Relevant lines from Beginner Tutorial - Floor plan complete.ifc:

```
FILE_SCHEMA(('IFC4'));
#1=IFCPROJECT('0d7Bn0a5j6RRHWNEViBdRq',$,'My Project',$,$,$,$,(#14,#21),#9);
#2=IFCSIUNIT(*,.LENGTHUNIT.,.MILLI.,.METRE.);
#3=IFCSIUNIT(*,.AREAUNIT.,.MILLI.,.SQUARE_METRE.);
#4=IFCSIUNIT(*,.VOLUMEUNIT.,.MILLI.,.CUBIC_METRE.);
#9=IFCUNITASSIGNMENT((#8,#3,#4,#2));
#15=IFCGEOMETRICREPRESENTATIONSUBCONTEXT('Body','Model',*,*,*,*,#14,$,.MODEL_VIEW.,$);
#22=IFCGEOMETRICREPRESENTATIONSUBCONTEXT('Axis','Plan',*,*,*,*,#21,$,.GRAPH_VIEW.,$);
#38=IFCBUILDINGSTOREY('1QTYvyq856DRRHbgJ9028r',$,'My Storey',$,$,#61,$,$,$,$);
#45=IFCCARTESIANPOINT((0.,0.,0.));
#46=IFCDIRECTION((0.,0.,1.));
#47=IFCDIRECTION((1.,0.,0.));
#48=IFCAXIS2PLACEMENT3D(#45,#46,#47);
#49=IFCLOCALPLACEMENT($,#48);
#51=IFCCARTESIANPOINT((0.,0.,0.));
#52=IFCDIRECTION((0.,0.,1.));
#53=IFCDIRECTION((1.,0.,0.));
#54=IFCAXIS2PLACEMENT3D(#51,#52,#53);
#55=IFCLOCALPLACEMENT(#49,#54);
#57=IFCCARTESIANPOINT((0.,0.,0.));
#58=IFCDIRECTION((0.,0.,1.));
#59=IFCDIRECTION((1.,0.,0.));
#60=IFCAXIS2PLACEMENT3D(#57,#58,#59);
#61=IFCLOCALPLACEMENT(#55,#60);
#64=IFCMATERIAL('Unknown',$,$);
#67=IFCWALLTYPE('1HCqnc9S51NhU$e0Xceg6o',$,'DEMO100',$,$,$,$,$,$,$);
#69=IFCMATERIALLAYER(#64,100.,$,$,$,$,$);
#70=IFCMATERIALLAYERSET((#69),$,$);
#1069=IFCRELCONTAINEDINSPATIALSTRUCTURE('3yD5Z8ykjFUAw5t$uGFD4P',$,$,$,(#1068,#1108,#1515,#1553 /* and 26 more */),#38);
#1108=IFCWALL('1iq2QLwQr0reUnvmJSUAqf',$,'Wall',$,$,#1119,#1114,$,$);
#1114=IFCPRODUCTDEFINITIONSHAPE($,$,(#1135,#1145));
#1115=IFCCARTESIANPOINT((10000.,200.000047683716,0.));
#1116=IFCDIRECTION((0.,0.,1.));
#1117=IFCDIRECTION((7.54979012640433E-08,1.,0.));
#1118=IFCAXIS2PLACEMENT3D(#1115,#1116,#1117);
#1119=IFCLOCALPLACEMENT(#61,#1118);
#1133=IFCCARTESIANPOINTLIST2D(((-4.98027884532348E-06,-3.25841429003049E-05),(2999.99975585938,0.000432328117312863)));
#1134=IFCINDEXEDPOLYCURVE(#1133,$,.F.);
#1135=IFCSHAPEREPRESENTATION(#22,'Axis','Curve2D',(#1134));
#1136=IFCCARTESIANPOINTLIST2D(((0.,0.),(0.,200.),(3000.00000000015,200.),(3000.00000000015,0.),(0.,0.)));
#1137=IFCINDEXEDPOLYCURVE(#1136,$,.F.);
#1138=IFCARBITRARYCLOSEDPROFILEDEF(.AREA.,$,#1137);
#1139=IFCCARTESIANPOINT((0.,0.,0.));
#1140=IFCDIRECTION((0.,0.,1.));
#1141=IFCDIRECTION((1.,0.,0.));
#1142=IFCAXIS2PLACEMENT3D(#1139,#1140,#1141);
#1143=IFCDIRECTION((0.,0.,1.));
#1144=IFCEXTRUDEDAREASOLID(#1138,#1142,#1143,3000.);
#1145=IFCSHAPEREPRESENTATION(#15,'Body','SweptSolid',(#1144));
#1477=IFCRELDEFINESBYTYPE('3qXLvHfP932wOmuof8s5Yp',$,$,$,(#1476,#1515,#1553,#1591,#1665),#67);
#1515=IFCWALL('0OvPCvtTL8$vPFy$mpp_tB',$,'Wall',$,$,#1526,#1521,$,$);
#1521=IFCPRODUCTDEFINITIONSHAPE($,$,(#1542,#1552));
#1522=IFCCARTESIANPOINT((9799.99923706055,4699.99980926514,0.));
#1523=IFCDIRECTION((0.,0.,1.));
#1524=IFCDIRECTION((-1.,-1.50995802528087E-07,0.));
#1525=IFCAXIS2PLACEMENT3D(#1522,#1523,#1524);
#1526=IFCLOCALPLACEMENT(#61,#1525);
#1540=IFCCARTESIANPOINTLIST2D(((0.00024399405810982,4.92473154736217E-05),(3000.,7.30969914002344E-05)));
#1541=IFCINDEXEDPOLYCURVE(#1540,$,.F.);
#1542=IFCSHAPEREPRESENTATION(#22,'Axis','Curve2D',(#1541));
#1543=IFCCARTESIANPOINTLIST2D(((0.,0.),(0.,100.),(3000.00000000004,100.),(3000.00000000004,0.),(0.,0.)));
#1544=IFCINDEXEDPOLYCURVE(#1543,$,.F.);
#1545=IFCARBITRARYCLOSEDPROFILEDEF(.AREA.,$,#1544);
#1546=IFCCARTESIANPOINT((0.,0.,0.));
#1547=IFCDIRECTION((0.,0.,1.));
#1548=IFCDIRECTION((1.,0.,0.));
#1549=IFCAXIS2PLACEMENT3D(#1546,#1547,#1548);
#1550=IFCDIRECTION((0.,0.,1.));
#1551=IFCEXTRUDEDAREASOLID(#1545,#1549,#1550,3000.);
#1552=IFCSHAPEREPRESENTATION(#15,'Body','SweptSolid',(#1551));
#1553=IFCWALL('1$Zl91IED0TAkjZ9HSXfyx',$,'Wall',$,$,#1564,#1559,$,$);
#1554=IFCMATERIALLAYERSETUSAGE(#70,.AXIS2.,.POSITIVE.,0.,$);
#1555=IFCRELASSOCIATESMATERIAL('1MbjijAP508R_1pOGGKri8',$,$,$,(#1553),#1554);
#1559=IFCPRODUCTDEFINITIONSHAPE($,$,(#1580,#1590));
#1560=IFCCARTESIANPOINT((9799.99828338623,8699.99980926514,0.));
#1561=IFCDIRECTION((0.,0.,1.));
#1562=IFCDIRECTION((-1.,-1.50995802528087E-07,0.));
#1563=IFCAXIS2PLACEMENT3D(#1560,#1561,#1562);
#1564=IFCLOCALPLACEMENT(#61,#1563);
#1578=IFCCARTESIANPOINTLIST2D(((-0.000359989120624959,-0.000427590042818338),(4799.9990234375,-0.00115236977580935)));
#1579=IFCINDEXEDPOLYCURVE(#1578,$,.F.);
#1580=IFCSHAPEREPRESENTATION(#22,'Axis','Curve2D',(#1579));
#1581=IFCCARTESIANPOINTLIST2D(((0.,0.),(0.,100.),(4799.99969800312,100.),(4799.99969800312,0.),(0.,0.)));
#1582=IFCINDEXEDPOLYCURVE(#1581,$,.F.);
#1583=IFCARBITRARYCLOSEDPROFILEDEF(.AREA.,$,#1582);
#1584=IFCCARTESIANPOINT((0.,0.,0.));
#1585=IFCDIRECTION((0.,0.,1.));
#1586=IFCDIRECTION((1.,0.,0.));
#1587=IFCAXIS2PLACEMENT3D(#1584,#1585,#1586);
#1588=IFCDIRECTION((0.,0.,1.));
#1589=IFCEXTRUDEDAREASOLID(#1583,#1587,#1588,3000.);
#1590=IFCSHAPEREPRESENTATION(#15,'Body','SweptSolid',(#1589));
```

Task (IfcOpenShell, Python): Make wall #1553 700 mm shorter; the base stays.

```python
import ifcopenshell
import ifcopenshell.geom
import ifcopenshell.util.representation
import ifcopenshell.util.shape

model = ifcopenshell.open("Beginner Tutorial - Floor plan complete.ifc")
settings = ifcopenshell.geom.settings()


def volume(element):
    """Net volume in cubic metres, openings subtracted."""
    shape = ifcopenshell.geom.create_shape(settings, element)
    return ifcopenshell.util.shape.get_volume(shape.geometry)


wall = model.by_id(1553)
before = volume(wall)

body = ifcopenshell.util.representation.get_representation(wall, "Model", "Body")
solid = body.Items[0]
old_height = solid.Depth
solid.Depth -= 700.0
after = volume(wall)

print(f"height {old_height:g} -> {solid.Depth:g}, volume {before:.3f} -> {after:.3f} m3")

model.write("Beginner Tutorial - Floor plan complete_edited.ifc")
```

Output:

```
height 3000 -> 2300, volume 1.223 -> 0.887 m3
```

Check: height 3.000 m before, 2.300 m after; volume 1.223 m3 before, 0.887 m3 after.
